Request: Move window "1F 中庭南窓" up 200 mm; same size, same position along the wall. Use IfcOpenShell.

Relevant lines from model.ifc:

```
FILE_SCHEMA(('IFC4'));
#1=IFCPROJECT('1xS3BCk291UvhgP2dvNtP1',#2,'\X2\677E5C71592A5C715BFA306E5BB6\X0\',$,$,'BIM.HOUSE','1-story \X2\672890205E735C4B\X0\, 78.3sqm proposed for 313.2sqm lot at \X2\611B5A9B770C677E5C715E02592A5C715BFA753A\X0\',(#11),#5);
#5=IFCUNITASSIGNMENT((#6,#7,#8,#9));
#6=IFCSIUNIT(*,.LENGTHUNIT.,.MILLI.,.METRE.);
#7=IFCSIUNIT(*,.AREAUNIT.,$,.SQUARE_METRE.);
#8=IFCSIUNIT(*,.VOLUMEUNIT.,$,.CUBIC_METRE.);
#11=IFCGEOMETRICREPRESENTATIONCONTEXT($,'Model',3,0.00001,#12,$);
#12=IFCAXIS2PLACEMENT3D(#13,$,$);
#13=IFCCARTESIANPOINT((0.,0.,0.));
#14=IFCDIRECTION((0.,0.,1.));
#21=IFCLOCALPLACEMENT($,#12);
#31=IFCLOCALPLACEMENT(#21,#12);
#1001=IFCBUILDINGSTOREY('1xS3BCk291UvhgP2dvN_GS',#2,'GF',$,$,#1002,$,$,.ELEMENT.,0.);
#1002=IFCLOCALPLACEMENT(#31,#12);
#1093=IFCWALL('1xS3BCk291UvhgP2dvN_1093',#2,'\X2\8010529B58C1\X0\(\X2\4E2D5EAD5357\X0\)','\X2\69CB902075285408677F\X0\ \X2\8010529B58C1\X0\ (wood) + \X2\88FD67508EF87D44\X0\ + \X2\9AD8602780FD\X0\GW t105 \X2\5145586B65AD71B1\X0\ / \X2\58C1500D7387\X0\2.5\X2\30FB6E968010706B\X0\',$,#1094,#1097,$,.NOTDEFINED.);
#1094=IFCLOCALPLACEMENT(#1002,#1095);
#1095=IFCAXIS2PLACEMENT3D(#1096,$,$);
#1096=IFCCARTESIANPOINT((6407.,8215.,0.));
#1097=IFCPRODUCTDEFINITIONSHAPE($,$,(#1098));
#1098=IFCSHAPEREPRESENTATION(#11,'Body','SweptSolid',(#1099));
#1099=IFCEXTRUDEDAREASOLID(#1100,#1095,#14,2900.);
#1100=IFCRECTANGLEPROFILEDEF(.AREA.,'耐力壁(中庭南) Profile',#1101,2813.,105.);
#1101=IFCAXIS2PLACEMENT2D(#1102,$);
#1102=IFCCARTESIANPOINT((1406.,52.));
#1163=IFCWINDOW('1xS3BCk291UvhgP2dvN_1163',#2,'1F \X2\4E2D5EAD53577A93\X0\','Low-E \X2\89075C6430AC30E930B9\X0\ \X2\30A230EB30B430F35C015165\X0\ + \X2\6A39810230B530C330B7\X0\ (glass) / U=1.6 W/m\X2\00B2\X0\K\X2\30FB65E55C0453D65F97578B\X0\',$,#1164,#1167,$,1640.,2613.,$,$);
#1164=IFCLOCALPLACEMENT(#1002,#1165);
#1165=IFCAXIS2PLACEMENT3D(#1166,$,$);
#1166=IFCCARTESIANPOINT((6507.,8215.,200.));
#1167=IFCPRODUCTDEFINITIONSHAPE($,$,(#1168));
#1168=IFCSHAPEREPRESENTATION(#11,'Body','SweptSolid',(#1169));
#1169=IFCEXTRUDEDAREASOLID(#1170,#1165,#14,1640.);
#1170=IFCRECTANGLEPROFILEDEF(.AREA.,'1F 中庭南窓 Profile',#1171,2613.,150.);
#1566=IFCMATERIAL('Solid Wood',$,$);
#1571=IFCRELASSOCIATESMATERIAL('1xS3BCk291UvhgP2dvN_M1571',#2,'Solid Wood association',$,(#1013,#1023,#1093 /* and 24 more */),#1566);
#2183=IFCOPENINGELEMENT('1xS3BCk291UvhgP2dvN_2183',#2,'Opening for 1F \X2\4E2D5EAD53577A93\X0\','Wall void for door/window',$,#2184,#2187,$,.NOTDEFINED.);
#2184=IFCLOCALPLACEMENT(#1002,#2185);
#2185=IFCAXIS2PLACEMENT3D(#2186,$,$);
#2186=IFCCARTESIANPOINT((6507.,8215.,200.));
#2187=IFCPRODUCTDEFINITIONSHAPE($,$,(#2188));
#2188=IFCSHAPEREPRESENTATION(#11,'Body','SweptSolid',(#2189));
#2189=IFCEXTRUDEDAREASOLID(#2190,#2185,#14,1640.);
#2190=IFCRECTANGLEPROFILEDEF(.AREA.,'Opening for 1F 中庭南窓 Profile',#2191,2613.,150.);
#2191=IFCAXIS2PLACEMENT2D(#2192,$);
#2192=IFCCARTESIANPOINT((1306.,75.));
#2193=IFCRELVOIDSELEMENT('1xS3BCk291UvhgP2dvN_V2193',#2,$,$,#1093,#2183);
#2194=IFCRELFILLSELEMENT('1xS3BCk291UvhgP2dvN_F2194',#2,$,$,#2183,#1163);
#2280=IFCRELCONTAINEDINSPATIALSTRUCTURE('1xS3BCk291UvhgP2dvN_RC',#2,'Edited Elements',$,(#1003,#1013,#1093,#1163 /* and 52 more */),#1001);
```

```python
import numpy as np
import ifcopenshell
import ifcopenshell.api.geometry
import ifcopenshell.util.placement
import ifcopenshell.util.unit

model = ifcopenshell.open("model.ifc")
unit_scale = ifcopenshell.util.unit.calculate_unit_scale(model)

window = model.by_guid("1xS3BCk291UvhgP2dvN_1163")
opening = window.FillsVoids[0].RelatingOpeningElement
dz = 0.2 / unit_scale

shift = np.array([0.0, 0.0, dz])
# The window is not placed relative to its opening, so move both.
for product in (opening, window):
    matrix = ifcopenshell.util.placement.get_local_placement(product.ObjectPlacement)
    matrix[:3, 3] += shift
    ifcopenshell.api.geometry.edit_object_placement(model, product=product, matrix=matrix, is_si=False)

print(f"moved by {dz * unit_scale:+.3f} m")

model.write("model_rev.ifc")
```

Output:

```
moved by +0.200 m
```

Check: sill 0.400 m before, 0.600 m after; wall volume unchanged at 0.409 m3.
